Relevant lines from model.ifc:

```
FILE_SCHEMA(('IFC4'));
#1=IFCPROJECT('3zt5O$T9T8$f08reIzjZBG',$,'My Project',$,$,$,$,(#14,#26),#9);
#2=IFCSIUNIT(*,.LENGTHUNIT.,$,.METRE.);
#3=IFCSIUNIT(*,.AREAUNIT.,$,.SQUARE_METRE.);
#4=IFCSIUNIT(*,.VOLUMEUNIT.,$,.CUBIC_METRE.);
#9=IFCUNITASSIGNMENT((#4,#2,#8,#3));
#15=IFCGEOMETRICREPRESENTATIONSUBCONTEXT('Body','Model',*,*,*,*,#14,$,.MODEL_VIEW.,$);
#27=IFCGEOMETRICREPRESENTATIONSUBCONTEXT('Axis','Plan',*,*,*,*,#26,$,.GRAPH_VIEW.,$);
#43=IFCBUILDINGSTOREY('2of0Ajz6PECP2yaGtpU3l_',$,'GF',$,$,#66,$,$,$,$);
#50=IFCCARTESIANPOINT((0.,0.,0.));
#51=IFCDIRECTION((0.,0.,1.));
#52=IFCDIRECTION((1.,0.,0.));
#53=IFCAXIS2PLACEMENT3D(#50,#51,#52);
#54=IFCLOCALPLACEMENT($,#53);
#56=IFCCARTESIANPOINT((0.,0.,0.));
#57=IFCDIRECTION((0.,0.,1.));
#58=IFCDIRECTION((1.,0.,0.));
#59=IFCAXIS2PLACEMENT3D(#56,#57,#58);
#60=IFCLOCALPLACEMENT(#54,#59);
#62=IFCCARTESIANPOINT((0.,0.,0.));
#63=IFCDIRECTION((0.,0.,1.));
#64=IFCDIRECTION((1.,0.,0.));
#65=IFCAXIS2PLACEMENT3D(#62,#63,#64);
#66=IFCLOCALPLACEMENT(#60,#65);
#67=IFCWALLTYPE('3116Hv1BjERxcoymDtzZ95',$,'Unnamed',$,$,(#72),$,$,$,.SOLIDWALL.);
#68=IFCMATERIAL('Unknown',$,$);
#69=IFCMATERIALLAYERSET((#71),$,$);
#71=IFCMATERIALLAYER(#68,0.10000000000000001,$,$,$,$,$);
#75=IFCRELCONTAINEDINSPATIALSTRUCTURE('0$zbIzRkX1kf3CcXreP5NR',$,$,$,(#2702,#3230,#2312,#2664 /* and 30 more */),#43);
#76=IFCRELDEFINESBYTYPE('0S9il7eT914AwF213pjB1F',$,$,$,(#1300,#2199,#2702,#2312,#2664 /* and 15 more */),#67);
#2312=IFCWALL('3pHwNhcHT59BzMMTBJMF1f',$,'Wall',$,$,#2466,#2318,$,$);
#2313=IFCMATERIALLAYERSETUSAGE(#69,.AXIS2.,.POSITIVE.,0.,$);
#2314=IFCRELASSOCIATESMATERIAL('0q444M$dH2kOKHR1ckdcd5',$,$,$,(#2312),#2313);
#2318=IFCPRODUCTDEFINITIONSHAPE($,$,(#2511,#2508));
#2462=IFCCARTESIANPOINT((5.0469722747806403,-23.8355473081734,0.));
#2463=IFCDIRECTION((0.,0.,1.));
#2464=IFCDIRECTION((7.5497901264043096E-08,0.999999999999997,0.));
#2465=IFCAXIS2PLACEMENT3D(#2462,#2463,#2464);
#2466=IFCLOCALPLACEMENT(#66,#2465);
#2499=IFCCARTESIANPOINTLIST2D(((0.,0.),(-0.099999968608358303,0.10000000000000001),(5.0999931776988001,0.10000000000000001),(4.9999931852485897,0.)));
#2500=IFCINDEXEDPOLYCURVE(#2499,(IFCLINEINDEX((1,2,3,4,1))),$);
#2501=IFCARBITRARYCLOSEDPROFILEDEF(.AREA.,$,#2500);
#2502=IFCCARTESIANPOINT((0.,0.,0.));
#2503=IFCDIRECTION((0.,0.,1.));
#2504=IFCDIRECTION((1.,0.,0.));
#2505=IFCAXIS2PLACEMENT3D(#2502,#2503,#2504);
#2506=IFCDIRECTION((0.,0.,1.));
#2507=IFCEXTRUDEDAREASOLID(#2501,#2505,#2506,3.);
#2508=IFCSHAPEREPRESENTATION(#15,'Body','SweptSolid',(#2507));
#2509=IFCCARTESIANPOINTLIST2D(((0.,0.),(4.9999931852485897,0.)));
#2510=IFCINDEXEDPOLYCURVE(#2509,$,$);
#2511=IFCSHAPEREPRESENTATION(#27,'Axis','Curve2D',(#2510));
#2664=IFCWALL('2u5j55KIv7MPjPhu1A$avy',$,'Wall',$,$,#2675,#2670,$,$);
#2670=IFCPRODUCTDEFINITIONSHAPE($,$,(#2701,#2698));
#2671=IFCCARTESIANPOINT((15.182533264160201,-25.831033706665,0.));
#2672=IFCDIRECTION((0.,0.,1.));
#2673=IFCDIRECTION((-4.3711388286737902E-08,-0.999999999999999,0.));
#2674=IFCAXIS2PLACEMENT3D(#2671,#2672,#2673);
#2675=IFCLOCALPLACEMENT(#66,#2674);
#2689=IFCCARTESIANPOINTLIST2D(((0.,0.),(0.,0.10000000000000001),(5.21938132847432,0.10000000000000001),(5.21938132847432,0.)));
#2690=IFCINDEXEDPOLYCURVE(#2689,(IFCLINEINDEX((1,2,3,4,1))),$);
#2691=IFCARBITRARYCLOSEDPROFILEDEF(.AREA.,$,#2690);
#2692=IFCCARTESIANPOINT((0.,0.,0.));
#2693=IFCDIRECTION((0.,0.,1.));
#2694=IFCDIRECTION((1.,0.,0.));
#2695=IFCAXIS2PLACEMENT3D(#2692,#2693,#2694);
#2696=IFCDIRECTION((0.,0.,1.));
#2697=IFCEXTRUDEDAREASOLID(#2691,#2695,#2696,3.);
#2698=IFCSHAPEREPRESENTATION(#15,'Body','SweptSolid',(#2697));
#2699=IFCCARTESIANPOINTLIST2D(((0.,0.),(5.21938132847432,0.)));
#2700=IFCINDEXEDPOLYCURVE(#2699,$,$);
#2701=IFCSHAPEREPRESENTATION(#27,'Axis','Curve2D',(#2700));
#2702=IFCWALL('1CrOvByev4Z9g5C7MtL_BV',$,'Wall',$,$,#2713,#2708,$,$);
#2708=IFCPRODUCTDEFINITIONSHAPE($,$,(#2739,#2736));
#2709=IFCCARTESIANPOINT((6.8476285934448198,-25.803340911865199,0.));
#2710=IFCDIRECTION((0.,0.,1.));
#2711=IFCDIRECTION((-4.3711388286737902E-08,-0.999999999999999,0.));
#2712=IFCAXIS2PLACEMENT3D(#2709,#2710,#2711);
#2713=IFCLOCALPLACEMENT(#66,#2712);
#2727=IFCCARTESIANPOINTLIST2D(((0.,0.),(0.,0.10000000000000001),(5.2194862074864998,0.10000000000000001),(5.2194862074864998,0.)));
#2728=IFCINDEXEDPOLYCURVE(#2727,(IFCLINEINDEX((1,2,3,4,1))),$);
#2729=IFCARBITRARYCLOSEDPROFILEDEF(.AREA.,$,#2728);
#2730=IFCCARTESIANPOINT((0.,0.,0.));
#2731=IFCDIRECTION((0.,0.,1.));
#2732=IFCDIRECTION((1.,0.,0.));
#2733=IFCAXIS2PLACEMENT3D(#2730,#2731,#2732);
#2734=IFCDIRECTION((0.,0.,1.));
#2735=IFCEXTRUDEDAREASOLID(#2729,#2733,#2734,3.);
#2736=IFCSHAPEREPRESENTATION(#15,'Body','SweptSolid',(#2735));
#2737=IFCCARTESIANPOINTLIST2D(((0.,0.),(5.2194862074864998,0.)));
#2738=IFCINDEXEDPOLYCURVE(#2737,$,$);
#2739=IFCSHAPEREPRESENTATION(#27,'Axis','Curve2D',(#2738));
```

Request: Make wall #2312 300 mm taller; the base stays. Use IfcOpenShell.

```python
import ifcopenshell
import ifcopenshell.geom
import ifcopenshell.util.representation
import ifcopenshell.util.shape

model = ifcopenshell.open("model.ifc")
settings = ifcopenshell.geom.settings()


def volume(element):
    """Net volume in cubic metres, openings subtracted."""
    shape = ifcopenshell.geom.create_shape(settings, element)
    return ifcopenshell.util.shape.get_volume(shape.geometry)


wall = model.by_guid("3pHwNhcHT59BzMMTBJMF1f")
before = volume(wall)

body = ifcopenshell.util.representation.get_representation(wall, "Model", "Body")
solid = body.Items[0]
old_height = solid.Depth
solid.Depth += 0.3
after = volume(wall)

print(f"height {old_height:g} -> {solid.Depth:g}, volume {before:.3f} -> {after:.3f} m3")

model.write("model-out.ifc")
```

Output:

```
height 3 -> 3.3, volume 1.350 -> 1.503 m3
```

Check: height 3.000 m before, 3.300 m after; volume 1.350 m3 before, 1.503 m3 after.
